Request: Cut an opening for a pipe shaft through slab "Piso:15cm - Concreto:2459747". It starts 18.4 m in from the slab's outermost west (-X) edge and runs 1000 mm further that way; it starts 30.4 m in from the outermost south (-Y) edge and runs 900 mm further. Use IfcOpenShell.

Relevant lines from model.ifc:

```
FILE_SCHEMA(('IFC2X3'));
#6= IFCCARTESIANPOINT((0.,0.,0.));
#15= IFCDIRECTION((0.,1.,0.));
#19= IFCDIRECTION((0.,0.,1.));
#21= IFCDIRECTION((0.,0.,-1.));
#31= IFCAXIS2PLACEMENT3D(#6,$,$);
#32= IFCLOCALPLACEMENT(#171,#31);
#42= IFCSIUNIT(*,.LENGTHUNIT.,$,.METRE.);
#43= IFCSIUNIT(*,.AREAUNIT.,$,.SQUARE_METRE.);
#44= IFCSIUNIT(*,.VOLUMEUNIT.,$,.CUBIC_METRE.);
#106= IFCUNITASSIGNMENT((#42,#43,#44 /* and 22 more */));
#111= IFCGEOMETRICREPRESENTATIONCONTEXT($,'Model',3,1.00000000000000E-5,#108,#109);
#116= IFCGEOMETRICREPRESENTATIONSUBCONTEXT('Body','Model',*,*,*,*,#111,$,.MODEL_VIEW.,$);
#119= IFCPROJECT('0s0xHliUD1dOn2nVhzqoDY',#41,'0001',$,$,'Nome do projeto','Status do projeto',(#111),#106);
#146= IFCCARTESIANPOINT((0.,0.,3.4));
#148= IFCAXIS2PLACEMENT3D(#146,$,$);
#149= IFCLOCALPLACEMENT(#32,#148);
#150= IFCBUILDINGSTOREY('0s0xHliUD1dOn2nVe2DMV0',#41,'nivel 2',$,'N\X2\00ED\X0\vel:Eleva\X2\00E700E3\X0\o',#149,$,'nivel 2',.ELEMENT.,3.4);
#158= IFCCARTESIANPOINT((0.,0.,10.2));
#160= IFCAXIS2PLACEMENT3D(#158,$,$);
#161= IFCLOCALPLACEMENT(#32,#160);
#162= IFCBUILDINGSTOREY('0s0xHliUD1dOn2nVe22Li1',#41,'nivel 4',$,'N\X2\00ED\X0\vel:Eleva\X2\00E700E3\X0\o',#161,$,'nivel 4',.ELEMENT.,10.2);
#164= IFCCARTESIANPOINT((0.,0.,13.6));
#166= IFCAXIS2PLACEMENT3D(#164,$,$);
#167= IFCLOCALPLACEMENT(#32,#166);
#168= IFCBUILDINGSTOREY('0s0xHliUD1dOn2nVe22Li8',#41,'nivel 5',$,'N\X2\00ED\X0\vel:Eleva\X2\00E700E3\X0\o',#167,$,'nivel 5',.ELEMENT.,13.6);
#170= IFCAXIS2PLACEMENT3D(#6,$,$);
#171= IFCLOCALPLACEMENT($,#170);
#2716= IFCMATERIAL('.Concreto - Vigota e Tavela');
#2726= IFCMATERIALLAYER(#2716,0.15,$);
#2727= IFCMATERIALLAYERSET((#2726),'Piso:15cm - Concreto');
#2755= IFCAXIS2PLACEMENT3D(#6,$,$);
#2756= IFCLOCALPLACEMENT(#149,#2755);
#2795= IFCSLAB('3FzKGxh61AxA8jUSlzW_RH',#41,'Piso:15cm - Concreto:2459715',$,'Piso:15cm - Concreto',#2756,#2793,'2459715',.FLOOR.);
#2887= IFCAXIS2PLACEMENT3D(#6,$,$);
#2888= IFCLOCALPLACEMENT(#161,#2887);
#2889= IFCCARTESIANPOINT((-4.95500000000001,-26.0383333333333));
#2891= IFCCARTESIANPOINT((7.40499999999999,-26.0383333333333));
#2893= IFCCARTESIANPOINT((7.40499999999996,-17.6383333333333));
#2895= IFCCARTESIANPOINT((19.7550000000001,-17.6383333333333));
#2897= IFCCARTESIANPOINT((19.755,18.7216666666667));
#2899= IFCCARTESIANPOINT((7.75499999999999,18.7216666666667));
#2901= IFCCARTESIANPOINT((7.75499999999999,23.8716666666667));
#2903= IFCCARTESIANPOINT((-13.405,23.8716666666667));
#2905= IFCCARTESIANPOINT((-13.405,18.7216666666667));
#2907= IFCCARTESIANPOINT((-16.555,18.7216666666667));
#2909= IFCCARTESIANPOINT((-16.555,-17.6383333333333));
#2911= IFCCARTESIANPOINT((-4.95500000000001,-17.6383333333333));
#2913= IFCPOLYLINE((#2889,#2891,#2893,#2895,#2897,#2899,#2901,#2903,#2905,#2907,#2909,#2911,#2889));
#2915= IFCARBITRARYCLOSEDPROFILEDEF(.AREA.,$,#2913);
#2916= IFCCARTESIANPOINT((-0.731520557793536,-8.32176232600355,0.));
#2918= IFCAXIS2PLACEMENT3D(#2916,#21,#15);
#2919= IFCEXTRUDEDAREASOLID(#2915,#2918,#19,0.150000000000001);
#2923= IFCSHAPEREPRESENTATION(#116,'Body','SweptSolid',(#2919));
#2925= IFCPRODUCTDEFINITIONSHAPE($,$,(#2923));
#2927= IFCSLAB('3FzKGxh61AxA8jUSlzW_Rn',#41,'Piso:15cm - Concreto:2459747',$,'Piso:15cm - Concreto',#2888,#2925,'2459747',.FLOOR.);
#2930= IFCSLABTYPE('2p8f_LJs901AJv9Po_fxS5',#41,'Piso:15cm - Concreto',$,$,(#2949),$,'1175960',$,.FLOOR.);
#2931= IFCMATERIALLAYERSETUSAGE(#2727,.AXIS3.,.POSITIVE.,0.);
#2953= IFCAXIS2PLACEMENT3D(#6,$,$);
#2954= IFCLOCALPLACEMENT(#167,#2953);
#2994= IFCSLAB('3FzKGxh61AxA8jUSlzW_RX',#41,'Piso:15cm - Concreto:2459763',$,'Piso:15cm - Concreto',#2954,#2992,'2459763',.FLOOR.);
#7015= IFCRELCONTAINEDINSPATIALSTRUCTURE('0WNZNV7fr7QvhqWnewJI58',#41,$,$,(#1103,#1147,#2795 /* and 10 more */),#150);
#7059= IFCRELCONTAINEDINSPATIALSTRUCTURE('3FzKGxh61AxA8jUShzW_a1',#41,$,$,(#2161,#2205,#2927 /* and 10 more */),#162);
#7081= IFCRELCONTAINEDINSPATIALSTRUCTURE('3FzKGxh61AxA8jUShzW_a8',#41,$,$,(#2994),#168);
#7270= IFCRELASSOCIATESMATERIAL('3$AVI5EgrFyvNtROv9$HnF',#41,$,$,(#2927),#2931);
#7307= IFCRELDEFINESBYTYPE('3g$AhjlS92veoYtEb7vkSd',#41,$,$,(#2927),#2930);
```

```python
import numpy as np
import ifcopenshell
import ifcopenshell.api.feature
import ifcopenshell.api.geometry
import ifcopenshell.api.root
import ifcopenshell.geom
import ifcopenshell.util.placement
import ifcopenshell.util.representation
import ifcopenshell.util.shape
import ifcopenshell.util.unit

model = ifcopenshell.open("model.ifc")
unit_scale = ifcopenshell.util.unit.calculate_unit_scale(model)
settings = ifcopenshell.geom.settings()


def volume(element):
    """Net volume in cubic metres, openings subtracted."""
    shape = ifcopenshell.geom.create_shape(settings, element)
    return ifcopenshell.util.shape.get_volume(shape.geometry)


slab = model.by_guid("3FzKGxh61AxA8jUSlzW_Rn")
before = volume(slab)

# Extent in the slab's own axes, in metres. The edges named are its -X and -Y sides.
slab_shape = ifcopenshell.geom.create_shape(settings, slab)
vertices = ifcopenshell.util.shape.get_vertices(slab_shape.geometry)
x_min, y_min, bottom = vertices.min(axis=0)
top = vertices[:, 2].max()

opening = ifcopenshell.api.root.create_entity(model, ifc_class="IfcOpeningElement", name="Pipe shaft opening")
context = ifcopenshell.util.representation.get_context(model, "Model", "Body", "MODEL_VIEW")
width, depth = 1, 0.9
outline = [(0.0, 0.0), (width, 0.0), (width, depth), (0.0, depth), (0.0, 0.0)]
# Overshoot both faces by 50 mm so the cut is clean.
shape = ifcopenshell.api.geometry.add_slab_representation(
    model, context=context, depth=top - bottom + 0.1, polyline=outline
)
ifcopenshell.api.geometry.assign_representation(model, product=opening, representation=shape)

matrix = ifcopenshell.util.placement.get_local_placement(slab.ObjectPlacement)
matrix[:, 3] = matrix @ np.append(np.array([x_min + 18.4, y_min + 30.4, bottom - 0.05]) / unit_scale, 1.0)
ifcopenshell.api.geometry.edit_object_placement(model, product=opening, matrix=matrix, is_si=False)
ifcopenshell.api.feature.add_feature(model, feature=opening, element=slab)

after = volume(slab)

print(f"slab volume {before:.3f} -> {after:.3f} m3")

model.write("model_edited.ifc")
```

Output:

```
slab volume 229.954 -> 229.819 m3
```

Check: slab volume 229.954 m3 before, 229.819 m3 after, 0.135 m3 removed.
